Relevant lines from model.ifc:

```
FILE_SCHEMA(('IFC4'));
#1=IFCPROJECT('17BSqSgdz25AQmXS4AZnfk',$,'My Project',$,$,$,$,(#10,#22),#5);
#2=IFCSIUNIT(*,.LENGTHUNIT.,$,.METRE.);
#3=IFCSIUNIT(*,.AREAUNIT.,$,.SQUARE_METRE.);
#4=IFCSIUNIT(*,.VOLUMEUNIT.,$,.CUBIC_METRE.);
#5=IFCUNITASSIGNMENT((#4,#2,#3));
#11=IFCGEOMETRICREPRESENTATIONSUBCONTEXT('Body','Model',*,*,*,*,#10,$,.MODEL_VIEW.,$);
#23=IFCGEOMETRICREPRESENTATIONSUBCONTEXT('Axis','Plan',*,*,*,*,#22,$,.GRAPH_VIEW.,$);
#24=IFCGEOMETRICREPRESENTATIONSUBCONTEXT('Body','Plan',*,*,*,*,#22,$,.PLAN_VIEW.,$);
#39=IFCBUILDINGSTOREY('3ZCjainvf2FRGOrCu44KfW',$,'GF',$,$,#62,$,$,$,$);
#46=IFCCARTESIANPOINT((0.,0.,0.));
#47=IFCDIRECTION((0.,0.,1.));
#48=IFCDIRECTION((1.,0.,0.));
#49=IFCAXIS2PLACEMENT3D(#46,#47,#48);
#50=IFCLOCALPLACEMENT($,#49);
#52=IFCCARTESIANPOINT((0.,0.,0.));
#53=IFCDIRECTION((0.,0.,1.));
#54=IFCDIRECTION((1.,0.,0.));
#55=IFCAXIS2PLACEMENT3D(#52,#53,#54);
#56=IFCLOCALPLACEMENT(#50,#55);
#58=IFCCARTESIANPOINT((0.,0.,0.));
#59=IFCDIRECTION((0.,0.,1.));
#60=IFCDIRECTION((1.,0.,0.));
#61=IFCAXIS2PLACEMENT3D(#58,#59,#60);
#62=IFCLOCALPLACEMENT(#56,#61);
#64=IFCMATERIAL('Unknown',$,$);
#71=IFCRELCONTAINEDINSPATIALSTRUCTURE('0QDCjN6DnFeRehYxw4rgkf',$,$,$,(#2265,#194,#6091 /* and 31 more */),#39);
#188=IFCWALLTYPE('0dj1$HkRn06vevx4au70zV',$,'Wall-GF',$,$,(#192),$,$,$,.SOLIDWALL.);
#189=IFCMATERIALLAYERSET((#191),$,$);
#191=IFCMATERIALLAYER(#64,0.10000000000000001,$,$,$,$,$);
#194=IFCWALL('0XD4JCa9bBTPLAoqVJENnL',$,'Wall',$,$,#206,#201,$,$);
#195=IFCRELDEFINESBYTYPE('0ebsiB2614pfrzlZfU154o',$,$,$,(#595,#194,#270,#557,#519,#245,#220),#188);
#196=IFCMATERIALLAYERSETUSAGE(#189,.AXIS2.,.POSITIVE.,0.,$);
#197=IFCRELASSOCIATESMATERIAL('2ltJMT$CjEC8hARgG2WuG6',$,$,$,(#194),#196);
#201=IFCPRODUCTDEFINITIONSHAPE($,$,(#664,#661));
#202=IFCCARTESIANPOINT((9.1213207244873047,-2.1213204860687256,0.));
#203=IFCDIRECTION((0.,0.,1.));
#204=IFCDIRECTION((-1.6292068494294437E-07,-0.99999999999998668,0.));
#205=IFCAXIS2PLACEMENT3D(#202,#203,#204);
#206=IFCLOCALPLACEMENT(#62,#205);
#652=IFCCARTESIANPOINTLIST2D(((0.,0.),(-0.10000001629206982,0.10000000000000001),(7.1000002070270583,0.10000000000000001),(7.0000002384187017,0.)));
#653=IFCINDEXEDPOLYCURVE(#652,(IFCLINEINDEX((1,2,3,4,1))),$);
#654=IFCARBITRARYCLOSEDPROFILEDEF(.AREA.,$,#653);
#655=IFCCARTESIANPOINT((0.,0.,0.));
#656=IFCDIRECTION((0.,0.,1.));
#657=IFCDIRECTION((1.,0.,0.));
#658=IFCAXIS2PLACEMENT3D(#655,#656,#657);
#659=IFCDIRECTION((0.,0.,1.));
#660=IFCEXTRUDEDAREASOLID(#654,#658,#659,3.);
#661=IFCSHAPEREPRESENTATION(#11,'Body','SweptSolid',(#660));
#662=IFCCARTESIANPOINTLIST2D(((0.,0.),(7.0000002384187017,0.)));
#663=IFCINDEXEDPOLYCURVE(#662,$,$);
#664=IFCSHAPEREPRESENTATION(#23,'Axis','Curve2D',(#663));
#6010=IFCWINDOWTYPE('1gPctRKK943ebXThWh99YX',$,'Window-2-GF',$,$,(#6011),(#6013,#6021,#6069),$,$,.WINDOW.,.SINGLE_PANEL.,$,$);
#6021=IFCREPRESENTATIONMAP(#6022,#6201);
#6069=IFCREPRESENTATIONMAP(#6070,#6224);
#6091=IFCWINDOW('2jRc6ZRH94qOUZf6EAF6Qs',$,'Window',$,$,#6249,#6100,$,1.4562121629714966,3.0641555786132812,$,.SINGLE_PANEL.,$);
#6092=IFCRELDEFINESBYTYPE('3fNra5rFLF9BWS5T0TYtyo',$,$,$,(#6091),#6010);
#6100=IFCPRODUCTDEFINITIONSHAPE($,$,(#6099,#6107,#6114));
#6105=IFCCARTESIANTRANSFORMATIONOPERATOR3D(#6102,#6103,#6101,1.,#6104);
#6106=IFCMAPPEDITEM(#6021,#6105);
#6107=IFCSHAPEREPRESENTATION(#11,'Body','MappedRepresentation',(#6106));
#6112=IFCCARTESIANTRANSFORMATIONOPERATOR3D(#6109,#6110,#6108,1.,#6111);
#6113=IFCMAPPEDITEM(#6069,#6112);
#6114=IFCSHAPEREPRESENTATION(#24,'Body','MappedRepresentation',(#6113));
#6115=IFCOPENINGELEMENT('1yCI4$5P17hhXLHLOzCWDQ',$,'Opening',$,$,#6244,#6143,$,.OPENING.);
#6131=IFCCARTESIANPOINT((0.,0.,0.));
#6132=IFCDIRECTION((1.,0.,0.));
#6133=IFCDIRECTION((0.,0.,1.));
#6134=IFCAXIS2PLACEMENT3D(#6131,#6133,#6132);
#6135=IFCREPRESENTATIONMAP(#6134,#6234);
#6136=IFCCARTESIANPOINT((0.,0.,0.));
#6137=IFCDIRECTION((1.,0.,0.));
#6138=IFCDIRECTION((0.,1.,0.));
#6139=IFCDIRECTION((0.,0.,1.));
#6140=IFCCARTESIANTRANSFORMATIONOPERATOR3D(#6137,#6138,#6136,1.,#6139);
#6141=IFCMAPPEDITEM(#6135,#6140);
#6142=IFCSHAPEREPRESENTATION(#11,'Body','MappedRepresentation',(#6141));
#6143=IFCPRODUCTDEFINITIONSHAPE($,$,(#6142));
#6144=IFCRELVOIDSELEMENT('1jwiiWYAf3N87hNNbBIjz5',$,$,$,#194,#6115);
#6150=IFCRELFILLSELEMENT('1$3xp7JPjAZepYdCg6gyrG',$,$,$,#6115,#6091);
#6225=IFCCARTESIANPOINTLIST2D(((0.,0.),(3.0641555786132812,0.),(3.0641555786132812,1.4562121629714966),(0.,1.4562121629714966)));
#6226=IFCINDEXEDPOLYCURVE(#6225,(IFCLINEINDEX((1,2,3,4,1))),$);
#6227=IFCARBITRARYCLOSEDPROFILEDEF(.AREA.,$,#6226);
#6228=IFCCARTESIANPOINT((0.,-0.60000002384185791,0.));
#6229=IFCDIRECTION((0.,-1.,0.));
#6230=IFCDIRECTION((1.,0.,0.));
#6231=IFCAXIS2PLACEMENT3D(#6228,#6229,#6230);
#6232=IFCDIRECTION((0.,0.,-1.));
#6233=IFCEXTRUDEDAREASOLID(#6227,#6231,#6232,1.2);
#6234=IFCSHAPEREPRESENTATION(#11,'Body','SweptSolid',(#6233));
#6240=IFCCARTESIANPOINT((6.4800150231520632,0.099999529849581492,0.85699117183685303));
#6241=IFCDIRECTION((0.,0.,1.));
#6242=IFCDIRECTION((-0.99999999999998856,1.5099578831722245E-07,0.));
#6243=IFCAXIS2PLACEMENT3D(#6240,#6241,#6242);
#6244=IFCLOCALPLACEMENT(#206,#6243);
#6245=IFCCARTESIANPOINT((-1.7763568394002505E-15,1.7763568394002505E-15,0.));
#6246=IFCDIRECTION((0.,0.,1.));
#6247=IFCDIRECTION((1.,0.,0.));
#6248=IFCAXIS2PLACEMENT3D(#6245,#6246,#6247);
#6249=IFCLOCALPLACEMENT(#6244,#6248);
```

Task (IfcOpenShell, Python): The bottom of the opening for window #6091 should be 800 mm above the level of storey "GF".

```python
import numpy as np
import ifcopenshell
import ifcopenshell.api.geometry
import ifcopenshell.geom
import ifcopenshell.util.element
import ifcopenshell.util.placement
import ifcopenshell.util.shape
import ifcopenshell.util.unit

model = ifcopenshell.open("model.ifc")
unit_scale = ifcopenshell.util.unit.calculate_unit_scale(model)

window = model.by_guid("2jRc6ZRH94qOUZf6EAF6Qs")
opening = window.FillsVoids[0].RelatingOpeningElement
storey = ifcopenshell.util.element.get_container(window, ifc_class="IfcBuildingStorey")
level = ifcopenshell.util.placement.get_local_placement(storey.ObjectPlacement)[2, 3]

# The opening's origin need not be at the sill, so measure its lowest point.
shape = ifcopenshell.geom.create_shape(ifcopenshell.geom.settings(), opening)
bottom = ifcopenshell.util.shape.get_shape_bottom_elevation(shape, shape.geometry) / unit_scale
dz = level + 0.8 / unit_scale - bottom

shift = np.array([0.0, 0.0, dz])
# The window is placed relative to its opening, so it follows when the opening moves.
matrix = ifcopenshell.util.placement.get_local_placement(opening.ObjectPlacement)
matrix[:3, 3] += shift
ifcopenshell.api.geometry.edit_object_placement(
    model, product=opening, matrix=matrix, is_si=False, should_transform_children=True
)

print(f"moved by {dz * unit_scale:+.3f} m")

model.write("model_rev.ifc")
```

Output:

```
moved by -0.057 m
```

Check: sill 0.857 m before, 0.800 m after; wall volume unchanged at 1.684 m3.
